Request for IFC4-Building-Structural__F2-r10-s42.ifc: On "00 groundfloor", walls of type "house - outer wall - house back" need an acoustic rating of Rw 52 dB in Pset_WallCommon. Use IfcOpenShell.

First a look at what the model holds.

```python
import ifcopenshell
import ifcopenshell.util.element

model = ifcopenshell.open("IFC4-Building-Structural__F2-r10-s42.ifc")
print(model.schema)
storey = next(s for s in model.by_type("IfcBuildingStorey") if s.Name == "00 groundfloor")
walls = [e for e in ifcopenshell.util.element.get_decomposition(storey) if e.is_a("IfcWall")]
seen = {}
for e in walls:
    element_type = ifcopenshell.util.element.get_type(e)
    key = (element_type.Name if element_type != e and element_type else None, ifcopenshell.util.element.get_pset(e, "Pset_WallCommon", "AcousticRating"))
    seen[key] = seen.get(key, 0) + 1
for (name, value), count in sorted(seen.items(), key=str):
    print(count, "x", name, "|", value)
```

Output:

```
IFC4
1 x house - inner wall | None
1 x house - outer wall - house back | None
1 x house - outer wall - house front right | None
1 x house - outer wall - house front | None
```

```python
import ifcopenshell
import ifcopenshell.api.pset
import ifcopenshell.util.element

model = ifcopenshell.open("IFC4-Building-Structural__F2-r10-s42.ifc")

storey = next(s for s in model.by_type("IfcBuildingStorey") if s.Name == "00 groundfloor")
walls = [e for e in ifcopenshell.util.element.get_decomposition(storey) if e.is_a("IfcWall")]

count = 0
for e in walls:
    element_type = ifcopenshell.util.element.get_type(e)
    if element_type in (None, e) or element_type.Name != "house - outer wall - house back":
        continue
    # add_pset returns the element's existing set when there is one.
    pset = ifcopenshell.api.pset.add_pset(model, product=e, name="Pset_WallCommon")
    ifcopenshell.api.pset.edit_pset(model, pset=pset, properties={"AcousticRating": "Rw 52 dB"})
    count += 1

print(count, "walls updated")

model.write("IFC4-Building-Structural__F2-r10-s42_edited.ifc")
```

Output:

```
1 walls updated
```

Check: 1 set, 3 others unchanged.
